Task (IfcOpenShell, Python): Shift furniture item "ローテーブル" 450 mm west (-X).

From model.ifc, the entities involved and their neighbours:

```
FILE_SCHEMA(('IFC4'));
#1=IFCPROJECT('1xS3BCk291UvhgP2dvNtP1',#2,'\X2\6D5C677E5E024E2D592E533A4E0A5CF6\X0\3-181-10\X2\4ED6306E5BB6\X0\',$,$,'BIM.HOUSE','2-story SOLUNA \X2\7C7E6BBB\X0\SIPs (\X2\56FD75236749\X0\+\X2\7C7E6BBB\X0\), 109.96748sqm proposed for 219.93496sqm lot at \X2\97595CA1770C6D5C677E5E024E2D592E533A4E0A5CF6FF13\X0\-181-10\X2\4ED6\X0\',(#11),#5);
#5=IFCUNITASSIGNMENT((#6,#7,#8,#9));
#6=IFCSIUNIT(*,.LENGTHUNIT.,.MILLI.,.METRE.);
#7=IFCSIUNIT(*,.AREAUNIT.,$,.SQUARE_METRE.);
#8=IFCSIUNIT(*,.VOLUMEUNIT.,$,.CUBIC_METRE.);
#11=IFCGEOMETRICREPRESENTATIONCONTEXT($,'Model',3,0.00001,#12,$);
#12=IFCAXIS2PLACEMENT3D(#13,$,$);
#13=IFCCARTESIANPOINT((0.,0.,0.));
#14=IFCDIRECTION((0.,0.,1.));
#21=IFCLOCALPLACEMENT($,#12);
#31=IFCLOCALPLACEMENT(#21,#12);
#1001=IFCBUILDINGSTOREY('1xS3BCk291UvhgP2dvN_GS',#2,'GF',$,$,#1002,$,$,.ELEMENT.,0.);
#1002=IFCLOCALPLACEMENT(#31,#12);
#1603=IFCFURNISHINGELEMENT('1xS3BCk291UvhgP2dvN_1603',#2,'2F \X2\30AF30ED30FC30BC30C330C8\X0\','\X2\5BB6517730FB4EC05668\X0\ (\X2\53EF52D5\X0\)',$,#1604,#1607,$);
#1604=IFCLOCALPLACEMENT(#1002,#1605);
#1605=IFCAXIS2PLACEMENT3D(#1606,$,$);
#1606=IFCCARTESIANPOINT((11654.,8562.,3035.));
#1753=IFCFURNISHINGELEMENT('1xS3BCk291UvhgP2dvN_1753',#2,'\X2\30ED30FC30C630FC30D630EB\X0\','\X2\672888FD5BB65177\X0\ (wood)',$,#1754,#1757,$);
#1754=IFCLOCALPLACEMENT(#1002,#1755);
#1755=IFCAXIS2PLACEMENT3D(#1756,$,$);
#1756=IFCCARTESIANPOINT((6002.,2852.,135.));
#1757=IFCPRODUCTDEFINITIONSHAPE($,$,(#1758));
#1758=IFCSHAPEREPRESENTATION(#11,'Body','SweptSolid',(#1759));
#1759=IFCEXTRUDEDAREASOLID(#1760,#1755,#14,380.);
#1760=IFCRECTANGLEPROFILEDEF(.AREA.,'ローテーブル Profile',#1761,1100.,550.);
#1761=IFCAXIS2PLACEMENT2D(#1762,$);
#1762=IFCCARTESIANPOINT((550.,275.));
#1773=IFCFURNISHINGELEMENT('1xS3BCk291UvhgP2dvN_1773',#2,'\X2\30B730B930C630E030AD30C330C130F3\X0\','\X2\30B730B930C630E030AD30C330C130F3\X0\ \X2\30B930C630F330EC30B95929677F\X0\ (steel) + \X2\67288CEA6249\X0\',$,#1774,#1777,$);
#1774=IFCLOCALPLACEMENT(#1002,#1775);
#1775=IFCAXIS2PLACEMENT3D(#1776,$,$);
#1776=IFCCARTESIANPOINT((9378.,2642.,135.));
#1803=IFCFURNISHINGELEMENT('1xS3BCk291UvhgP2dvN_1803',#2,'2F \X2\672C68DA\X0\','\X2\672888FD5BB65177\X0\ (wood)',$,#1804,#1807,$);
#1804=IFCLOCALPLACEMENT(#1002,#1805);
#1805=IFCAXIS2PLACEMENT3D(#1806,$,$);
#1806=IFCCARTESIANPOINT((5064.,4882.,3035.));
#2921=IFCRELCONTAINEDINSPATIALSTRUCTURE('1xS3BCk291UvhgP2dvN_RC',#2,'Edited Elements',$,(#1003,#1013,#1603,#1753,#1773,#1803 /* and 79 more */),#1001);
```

```python
import ifcopenshell
import ifcopenshell.api.geometry
import ifcopenshell.util.placement

model = ifcopenshell.open("model.ifc")

item = model.by_id(1753)
matrix = ifcopenshell.util.placement.get_local_placement(item.ObjectPlacement)
matrix[0, 3] -= 450.0
ifcopenshell.api.geometry.edit_object_placement(model, product=item, matrix=matrix, is_si=False)

print(ifcopenshell.util.placement.get_local_placement(item.ObjectPlacement).round(3) + 0.0)

model.write("model_v2.ifc")
```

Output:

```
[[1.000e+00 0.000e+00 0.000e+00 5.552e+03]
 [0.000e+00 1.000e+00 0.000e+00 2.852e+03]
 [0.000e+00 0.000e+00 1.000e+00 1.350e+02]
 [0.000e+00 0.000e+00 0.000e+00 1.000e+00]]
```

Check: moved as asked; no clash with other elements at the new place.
